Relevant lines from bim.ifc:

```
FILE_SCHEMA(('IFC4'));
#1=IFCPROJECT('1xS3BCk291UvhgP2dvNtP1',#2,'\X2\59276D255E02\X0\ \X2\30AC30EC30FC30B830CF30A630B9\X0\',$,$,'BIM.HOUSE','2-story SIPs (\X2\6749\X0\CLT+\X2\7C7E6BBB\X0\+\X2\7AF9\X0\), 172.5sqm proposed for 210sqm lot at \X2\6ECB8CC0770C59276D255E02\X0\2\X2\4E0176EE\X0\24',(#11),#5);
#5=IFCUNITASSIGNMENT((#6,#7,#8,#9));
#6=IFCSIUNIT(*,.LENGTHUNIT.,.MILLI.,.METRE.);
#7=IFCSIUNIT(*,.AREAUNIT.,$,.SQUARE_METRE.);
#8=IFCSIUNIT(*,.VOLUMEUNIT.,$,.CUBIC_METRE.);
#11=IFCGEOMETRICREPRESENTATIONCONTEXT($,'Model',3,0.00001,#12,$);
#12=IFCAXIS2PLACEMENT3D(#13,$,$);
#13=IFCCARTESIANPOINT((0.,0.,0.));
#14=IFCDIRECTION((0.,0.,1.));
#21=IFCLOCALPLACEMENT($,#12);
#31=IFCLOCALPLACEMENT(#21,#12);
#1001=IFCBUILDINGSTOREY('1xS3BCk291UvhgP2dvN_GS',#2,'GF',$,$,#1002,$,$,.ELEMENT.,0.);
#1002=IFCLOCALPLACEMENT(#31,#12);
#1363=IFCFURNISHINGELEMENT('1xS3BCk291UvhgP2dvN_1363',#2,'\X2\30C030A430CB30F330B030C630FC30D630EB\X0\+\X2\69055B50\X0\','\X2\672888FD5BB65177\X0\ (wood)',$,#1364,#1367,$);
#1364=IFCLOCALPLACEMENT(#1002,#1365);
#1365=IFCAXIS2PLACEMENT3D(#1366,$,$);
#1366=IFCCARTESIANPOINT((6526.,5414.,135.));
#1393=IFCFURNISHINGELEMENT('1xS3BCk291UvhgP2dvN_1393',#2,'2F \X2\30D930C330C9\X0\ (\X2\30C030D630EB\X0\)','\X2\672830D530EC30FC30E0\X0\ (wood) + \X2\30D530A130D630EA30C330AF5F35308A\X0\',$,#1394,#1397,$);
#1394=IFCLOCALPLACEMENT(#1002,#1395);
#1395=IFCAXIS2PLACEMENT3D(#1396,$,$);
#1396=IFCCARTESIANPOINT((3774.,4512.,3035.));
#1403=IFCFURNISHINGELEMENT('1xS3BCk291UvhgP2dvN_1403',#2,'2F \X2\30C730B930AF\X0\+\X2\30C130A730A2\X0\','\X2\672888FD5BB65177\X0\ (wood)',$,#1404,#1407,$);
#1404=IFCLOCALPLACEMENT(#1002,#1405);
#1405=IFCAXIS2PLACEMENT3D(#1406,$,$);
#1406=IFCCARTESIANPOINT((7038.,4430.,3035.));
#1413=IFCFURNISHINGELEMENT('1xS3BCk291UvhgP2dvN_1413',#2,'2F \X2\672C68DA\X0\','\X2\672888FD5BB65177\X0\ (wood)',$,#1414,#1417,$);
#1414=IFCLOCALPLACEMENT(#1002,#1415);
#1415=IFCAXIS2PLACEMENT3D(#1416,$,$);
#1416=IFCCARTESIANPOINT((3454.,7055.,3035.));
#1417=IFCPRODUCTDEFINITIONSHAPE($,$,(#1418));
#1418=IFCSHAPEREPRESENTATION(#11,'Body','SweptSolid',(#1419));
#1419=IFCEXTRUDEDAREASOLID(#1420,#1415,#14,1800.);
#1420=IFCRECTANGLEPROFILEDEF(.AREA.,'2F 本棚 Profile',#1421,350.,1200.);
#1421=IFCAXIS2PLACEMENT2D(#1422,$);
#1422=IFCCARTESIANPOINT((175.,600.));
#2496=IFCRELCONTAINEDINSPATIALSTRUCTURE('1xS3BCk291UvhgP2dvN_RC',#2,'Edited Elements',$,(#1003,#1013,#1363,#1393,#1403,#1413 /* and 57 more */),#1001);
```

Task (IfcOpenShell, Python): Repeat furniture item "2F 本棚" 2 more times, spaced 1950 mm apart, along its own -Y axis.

```python
import ifcopenshell
import ifcopenshell.api.geometry
import ifcopenshell.api.root
import ifcopenshell.util.element
import ifcopenshell.util.placement

model = ifcopenshell.open("bim.ifc")


def reuse_history(source, copy):
    """copy_class also copies each property set's owner history, people and application; keep the originals."""
    for rel in copy.IsDefinedBy:
        if rel.is_a("IfcRelDefinesByProperties") and (history := rel.RelatingPropertyDefinition.OwnerHistory):
            rel.RelatingPropertyDefinition.OwnerHistory = source.OwnerHistory
            ifcopenshell.util.element.remove_deep2(model, history)


source = model.by_id(1413)
base = ifcopenshell.util.placement.get_local_placement(source.ObjectPlacement)
step = -base[:3, 1] * 1950.0

for i in range(1, 3):
    copy = ifcopenshell.api.root.copy_class(model, product=source)
    copy.Representation = ifcopenshell.util.element.copy_deep(
        model, source.Representation, exclude=["IfcGeometricRepresentationContext", "IfcRepresentationMap"]
    )
    reuse_history(source, copy)
    matrix = base.copy()
    matrix[:3, 3] += i * step
    print("added at", matrix[:3, 3].round(3) + 0.0)
    ifcopenshell.api.geometry.edit_object_placement(model, product=copy, matrix=matrix, is_si=False)

model.write("bim_edited.ifc")
```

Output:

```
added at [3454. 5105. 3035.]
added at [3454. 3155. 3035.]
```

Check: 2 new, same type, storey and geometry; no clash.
